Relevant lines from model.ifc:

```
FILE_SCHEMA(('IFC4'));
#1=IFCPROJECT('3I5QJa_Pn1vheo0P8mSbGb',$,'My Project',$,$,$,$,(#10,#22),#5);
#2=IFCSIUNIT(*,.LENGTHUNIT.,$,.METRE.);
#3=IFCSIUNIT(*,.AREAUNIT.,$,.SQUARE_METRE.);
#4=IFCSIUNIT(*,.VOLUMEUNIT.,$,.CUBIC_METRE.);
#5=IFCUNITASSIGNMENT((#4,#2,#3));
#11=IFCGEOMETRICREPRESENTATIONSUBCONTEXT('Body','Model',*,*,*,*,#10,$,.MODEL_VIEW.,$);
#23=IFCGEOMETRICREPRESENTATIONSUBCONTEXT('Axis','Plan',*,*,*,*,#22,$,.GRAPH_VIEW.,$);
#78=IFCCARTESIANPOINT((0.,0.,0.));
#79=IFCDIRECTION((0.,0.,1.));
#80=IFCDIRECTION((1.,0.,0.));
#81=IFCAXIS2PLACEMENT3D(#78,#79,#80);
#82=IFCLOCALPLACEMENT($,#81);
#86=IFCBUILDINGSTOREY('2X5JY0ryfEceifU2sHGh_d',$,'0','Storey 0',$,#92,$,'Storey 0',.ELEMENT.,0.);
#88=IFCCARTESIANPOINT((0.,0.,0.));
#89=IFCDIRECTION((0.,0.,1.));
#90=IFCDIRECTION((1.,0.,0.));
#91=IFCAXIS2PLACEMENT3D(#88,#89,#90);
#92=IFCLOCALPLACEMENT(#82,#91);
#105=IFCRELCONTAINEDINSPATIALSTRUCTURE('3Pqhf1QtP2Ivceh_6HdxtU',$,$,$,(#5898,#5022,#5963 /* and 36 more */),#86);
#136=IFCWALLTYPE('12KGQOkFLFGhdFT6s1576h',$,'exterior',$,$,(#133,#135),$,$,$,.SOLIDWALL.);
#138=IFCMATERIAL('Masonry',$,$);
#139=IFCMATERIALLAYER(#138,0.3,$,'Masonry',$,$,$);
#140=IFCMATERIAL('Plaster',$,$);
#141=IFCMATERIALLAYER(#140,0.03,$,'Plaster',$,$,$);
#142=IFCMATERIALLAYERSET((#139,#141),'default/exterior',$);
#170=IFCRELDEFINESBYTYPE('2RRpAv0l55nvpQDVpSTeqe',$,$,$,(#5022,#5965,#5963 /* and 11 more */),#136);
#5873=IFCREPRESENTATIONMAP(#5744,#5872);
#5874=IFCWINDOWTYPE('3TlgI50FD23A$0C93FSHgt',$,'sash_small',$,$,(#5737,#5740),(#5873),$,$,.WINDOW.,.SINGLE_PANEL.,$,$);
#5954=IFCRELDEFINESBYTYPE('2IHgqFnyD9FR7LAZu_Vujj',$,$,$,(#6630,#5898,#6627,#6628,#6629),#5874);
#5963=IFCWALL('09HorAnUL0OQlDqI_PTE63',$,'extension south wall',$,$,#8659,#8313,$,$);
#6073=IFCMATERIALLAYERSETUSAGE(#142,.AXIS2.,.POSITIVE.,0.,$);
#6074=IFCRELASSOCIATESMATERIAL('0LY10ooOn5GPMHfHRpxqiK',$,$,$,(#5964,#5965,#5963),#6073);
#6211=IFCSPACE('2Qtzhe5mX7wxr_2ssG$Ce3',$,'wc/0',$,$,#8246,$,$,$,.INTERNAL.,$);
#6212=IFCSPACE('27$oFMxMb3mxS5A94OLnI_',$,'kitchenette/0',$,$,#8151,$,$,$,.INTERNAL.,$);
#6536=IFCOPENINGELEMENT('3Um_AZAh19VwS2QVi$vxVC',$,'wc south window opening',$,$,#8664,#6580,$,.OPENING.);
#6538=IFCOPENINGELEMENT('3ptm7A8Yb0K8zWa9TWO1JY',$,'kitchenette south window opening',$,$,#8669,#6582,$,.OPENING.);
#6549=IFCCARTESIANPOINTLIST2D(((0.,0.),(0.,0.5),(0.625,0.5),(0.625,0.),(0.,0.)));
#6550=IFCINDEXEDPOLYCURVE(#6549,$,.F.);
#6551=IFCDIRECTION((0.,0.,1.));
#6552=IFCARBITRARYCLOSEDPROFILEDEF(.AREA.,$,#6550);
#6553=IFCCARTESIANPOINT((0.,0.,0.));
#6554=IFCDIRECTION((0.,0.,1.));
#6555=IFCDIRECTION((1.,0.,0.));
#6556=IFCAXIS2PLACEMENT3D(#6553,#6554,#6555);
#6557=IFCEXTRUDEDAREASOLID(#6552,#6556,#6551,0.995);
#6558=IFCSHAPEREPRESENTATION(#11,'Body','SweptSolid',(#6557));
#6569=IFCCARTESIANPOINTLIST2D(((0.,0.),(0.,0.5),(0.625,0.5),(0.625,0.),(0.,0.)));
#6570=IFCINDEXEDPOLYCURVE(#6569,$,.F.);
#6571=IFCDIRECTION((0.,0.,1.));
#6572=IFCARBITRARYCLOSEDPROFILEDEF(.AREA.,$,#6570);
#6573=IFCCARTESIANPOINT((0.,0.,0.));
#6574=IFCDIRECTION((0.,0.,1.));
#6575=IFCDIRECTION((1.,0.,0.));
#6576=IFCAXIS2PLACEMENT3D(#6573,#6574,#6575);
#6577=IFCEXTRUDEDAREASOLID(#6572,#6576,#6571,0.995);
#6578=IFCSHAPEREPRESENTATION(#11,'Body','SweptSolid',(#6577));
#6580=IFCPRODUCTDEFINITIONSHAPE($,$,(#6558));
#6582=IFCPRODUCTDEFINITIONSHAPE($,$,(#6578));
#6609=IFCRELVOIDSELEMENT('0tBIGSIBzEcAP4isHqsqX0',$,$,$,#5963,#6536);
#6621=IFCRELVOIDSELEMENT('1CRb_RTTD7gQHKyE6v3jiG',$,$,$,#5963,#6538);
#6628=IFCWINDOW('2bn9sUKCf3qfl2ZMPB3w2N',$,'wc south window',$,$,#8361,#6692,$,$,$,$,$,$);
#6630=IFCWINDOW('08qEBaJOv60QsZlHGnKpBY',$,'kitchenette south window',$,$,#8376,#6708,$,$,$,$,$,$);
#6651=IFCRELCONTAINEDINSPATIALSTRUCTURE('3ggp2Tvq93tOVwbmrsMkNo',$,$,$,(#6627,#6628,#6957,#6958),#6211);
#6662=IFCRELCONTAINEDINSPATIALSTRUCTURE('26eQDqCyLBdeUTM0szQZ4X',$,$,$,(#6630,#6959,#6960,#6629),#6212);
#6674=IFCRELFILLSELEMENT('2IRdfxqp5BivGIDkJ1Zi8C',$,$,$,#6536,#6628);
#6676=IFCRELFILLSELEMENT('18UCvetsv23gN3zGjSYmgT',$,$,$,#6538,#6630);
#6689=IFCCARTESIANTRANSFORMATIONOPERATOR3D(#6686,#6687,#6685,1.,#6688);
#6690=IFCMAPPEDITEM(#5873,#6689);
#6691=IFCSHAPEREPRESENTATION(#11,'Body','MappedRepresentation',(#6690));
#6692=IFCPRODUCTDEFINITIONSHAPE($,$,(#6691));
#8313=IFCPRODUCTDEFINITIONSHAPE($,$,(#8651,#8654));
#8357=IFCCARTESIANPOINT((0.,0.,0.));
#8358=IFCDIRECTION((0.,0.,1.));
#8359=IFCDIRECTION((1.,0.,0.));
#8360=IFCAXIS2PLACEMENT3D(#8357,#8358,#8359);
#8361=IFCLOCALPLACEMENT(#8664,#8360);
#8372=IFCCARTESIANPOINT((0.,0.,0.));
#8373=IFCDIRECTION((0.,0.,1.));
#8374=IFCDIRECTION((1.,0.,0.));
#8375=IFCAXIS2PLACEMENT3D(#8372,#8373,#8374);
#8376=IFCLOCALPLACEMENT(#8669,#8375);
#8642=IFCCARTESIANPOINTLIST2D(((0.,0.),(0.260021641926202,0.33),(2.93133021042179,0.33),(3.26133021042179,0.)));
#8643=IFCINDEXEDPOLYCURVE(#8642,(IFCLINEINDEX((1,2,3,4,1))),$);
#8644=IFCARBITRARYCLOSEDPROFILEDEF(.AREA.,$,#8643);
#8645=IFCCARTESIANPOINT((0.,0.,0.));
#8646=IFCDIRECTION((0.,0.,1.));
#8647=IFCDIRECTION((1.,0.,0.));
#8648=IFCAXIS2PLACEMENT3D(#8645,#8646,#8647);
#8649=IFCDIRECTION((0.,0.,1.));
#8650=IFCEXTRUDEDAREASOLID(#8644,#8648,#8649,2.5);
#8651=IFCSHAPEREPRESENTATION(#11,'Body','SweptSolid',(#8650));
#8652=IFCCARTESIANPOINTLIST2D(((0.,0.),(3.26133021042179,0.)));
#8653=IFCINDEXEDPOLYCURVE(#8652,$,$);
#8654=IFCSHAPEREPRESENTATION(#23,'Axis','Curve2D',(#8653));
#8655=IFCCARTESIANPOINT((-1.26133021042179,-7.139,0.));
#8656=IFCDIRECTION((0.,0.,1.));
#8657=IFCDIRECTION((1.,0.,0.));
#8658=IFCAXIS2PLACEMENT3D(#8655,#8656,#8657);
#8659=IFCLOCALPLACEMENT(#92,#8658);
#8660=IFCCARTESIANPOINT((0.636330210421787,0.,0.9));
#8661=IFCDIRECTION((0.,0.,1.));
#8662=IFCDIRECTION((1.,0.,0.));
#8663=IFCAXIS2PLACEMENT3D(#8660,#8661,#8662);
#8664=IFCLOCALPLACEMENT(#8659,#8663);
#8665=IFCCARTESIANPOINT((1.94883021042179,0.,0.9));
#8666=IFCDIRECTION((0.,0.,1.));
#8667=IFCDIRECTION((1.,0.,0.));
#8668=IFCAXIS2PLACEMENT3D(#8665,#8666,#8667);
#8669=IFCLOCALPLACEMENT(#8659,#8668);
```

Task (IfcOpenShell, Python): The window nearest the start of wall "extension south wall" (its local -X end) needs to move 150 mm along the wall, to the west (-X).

```python
import ifcopenshell
import ifcopenshell.api.geometry
import ifcopenshell.util.placement
import ifcopenshell.util.unit

model = ifcopenshell.open("model.ifc")
unit_scale = ifcopenshell.util.unit.calculate_unit_scale(model)

window = model.by_id(6628)
opening = window.FillsVoids[0].RelatingOpeningElement
wall = opening.VoidsElements[0].RelatingBuildingElement

wall_matrix = ifcopenshell.util.placement.get_local_placement(wall.ObjectPlacement)
shift = wall_matrix[:3, 0] * -0.15 / unit_scale
before = ifcopenshell.util.placement.get_local_placement(window.ObjectPlacement)[:3, 3].copy()

# The window is placed relative to its opening, so it follows when the opening moves.
matrix = ifcopenshell.util.placement.get_local_placement(opening.ObjectPlacement)
matrix[:3, 3] += shift
ifcopenshell.api.geometry.edit_object_placement(
    model, product=opening, matrix=matrix, is_si=False, should_transform_children=True
)

after = ifcopenshell.util.placement.get_local_placement(window.ObjectPlacement)[:3, 3]
print("window moved by", (after - before).round(3) + 0.0)

model.write("model_updated.ifc")
```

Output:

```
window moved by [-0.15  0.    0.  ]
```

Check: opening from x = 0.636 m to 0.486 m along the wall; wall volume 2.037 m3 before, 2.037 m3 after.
